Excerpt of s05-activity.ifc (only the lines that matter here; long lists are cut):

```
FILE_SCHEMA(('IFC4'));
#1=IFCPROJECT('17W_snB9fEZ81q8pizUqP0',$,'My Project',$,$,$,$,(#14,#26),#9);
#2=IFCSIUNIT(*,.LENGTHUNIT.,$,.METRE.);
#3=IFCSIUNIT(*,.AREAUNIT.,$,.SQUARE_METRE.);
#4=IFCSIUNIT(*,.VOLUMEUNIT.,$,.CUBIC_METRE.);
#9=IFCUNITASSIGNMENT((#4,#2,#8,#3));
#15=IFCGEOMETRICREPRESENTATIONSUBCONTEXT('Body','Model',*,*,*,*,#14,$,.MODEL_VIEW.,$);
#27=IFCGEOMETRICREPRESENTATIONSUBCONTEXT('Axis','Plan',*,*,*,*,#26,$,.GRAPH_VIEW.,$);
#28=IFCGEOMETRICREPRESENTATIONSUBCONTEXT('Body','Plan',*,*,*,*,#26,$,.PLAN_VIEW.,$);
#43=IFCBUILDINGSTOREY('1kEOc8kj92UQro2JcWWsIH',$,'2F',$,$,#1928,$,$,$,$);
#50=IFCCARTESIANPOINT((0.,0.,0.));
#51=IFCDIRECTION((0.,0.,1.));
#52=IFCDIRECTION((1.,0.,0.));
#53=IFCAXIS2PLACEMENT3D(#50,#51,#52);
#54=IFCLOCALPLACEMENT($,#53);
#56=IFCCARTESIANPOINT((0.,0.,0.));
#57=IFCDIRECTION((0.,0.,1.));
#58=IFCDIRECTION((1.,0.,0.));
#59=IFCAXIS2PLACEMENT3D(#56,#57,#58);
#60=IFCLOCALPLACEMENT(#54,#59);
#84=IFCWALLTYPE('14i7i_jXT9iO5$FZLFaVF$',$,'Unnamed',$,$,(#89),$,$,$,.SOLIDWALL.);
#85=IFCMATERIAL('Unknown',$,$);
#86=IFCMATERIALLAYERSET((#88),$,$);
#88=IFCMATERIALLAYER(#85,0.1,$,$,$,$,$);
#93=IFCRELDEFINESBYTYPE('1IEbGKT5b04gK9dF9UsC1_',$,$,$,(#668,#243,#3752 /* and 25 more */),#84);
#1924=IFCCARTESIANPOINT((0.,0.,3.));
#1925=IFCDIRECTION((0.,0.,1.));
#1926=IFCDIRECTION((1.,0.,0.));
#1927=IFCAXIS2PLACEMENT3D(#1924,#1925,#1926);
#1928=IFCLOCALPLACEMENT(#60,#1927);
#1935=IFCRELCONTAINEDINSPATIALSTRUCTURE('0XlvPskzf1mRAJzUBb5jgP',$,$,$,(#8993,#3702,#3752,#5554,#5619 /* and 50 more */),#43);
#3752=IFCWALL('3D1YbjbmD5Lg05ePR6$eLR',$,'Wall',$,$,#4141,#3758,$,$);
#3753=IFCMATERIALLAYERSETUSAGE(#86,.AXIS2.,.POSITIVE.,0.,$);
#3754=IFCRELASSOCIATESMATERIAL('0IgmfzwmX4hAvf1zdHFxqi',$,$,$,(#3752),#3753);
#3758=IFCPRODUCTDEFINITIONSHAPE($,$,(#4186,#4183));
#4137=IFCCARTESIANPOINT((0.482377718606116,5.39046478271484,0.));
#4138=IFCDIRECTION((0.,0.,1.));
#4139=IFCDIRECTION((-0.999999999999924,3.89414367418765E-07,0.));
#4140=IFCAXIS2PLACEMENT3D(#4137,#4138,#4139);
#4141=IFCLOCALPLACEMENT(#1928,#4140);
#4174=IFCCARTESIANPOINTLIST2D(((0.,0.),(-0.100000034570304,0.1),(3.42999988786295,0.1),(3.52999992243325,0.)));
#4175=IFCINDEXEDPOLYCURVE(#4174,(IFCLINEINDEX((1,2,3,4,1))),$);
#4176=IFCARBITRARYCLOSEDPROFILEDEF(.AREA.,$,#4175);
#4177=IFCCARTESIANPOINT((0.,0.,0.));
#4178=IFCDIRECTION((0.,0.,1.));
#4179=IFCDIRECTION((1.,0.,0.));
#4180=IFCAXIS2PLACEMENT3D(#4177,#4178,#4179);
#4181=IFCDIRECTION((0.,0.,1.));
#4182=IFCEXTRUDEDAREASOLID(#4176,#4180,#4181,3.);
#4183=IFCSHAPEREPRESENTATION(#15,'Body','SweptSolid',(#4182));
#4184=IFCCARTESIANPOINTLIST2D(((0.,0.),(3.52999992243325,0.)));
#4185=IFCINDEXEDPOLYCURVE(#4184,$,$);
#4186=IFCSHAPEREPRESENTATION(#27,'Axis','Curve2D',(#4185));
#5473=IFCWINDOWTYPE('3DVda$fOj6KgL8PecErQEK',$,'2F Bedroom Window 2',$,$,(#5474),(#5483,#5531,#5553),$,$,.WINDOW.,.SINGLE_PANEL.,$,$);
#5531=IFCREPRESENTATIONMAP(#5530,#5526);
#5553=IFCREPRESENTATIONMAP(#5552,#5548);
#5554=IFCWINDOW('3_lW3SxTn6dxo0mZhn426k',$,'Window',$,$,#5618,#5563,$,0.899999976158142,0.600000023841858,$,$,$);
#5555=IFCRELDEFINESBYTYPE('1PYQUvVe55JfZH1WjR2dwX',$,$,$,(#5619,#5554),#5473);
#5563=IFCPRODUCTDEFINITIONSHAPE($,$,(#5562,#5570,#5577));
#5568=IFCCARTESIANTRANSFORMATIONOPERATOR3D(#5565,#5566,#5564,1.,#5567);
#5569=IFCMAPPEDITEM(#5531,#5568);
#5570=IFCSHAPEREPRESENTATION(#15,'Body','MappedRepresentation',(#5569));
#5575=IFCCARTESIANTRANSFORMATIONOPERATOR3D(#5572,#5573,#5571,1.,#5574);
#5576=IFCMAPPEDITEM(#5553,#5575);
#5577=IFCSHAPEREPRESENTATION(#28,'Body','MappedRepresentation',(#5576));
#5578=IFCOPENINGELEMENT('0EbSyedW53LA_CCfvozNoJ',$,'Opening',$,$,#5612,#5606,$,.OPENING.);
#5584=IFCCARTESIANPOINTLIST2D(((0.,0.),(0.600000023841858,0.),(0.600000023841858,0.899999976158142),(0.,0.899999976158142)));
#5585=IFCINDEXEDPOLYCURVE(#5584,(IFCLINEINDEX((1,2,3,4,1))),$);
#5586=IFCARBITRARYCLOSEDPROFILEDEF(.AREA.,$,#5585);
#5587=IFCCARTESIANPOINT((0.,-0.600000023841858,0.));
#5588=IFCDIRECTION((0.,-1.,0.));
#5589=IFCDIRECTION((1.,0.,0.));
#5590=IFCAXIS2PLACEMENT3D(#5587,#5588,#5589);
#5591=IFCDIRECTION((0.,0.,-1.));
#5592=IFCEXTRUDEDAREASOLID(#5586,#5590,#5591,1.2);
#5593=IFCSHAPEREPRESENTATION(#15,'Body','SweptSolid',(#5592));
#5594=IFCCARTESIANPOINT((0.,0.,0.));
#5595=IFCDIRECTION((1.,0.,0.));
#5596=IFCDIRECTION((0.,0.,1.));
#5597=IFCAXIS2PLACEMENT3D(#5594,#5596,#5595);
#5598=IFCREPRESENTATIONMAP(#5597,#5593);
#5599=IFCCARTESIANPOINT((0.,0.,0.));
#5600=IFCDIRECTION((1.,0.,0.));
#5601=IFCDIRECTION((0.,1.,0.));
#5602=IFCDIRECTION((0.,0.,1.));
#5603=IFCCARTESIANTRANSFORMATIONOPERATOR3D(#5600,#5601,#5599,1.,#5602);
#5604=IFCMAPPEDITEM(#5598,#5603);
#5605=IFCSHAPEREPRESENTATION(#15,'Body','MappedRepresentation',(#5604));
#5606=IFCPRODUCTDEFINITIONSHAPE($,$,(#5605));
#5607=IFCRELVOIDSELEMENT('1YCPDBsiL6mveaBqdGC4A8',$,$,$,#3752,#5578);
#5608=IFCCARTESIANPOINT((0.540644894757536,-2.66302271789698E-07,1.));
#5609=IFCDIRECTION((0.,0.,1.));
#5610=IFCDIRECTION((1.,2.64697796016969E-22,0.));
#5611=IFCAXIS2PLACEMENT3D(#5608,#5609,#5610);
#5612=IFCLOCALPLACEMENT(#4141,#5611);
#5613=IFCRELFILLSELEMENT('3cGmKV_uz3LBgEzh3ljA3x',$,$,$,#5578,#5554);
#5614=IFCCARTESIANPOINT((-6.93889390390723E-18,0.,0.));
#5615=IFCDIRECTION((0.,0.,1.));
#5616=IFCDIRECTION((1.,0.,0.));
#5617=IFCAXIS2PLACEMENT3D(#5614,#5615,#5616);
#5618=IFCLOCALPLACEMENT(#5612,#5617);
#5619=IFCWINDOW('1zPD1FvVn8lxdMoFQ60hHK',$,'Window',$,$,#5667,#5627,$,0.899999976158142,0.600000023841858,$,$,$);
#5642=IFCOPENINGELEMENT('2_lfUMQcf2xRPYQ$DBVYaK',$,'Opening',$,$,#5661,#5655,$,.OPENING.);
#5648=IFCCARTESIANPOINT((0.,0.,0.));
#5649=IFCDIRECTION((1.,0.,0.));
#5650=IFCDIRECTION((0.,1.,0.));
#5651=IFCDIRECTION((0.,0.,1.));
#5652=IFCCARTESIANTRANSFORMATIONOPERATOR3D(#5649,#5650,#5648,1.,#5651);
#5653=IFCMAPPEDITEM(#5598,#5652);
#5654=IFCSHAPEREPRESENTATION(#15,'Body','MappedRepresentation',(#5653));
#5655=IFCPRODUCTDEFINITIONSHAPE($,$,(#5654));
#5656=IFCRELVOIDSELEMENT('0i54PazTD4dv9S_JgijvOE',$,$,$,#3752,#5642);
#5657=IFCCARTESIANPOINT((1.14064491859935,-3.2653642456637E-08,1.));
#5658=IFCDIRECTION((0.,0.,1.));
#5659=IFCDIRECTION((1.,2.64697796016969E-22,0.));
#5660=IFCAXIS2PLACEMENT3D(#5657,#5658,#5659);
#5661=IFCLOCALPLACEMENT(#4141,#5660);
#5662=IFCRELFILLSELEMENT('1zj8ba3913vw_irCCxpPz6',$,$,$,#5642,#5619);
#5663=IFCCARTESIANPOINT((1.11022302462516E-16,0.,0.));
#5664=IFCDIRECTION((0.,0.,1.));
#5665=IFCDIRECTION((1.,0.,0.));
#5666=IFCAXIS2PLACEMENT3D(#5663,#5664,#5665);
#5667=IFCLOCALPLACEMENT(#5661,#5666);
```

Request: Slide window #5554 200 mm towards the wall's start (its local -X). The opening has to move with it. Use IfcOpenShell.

```python
import ifcopenshell
import ifcopenshell.api.geometry
import ifcopenshell.util.placement

model = ifcopenshell.open("s05-activity.ifc")

window = model.by_guid("3_lW3SxTn6dxo0mZhn426k")
opening = window.FillsVoids[0].RelatingOpeningElement
wall = opening.VoidsElements[0].RelatingBuildingElement

wall_matrix = ifcopenshell.util.placement.get_local_placement(wall.ObjectPlacement)
shift = wall_matrix[:3, 0] * -0.2
before = ifcopenshell.util.placement.get_local_placement(window.ObjectPlacement)[:3, 3].copy()

# The window is placed relative to its opening, so it follows when the opening moves.
matrix = ifcopenshell.util.placement.get_local_placement(opening.ObjectPlacement)
matrix[:3, 3] += shift
ifcopenshell.api.geometry.edit_object_placement(
    model, product=opening, matrix=matrix, is_si=False, should_transform_children=True
)

after = ifcopenshell.util.placement.get_local_placement(window.ObjectPlacement)[:3, 3]
print("window moved by", (after - before).round(3) + 0.0)

model.write("s05-activity-out.ifc")
```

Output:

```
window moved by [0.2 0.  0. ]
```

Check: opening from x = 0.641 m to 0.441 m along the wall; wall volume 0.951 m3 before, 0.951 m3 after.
